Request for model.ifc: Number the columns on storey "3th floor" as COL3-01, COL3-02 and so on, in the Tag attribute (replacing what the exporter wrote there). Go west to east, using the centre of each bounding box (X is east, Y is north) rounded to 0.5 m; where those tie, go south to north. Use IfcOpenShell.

First a look at what the model holds.

```python
import ifcopenshell
import ifcopenshell.util.element
import ifcopenshell.util.placement

model = ifcopenshell.open("model.ifc")
print(model.schema)
storey = next(s for s in model.by_type("IfcBuildingStorey") if s.Name == "3th floor")
columns = [e for e in ifcopenshell.util.element.get_decomposition(storey) if e.is_a("IfcColumn")]
for e in sorted(columns, key=lambda e: e.id()):
    origin = ifcopenshell.util.placement.get_local_placement(e.ObjectPlacement)[:3, 3]
    print(e.id(), e.Tag, e.Name, origin.round(2) + 0.0, sep=" | ")
```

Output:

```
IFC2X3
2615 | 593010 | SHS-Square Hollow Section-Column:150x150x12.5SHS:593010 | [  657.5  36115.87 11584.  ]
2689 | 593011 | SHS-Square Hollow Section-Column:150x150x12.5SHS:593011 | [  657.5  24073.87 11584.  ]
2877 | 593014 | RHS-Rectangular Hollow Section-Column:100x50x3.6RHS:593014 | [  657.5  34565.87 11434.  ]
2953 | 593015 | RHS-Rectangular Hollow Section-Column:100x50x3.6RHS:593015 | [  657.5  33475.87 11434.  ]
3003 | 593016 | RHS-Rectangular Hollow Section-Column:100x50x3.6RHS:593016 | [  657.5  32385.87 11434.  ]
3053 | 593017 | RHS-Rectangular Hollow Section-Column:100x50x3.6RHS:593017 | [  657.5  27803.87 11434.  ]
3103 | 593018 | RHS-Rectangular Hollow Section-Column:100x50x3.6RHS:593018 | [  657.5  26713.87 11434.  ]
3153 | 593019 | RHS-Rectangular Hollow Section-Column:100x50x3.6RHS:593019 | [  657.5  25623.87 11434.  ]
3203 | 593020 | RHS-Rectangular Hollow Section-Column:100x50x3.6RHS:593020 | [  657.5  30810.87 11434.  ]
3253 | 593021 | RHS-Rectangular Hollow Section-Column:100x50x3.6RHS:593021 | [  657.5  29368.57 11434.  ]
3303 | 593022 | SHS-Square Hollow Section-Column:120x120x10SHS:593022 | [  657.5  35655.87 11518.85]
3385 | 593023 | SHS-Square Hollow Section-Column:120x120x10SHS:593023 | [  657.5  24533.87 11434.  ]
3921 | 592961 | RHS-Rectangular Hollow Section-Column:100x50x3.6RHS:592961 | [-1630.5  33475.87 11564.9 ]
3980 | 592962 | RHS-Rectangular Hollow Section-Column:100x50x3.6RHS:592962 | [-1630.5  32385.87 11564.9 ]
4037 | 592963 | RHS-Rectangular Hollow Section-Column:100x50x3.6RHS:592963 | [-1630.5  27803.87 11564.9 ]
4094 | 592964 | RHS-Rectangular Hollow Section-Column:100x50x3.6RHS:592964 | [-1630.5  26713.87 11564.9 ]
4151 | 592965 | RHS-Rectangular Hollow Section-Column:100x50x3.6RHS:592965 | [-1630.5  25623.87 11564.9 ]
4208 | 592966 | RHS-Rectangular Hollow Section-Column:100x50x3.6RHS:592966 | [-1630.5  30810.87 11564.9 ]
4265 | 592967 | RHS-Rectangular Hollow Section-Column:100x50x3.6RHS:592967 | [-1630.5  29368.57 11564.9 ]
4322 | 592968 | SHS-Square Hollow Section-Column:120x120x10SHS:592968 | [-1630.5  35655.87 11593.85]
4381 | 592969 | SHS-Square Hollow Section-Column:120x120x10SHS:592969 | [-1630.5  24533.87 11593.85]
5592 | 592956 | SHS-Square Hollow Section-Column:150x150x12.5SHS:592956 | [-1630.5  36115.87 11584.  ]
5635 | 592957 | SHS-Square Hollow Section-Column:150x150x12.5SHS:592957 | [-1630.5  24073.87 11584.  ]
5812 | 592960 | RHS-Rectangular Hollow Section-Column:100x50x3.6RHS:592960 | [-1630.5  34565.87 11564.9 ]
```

```python
import ifcopenshell
import ifcopenshell.geom
import ifcopenshell.util.element
import ifcopenshell.util.shape

model = ifcopenshell.open("model.ifc")
settings = ifcopenshell.geom.settings()
settings.set("use-world-coords", True)


def centre(element):
    shape = ifcopenshell.geom.create_shape(settings, element)
    return ifcopenshell.util.shape.get_bbox_centroid(shape.geometry)


storey = next(s for s in model.by_type("IfcBuildingStorey") if s.Name == "3th floor")
columns = [e for e in ifcopenshell.util.element.get_decomposition(storey) if e.is_a("IfcColumn")]

# Insertion points can sit at a corner or the storey origin, so sort by the geometry (in metres).
centres = {e: centre(e) for e in columns}
columns.sort(key=lambda e: (round(centres[e][0] / 0.5), centres[e][1]))

for i, e in enumerate(columns, start=1):
    number = f"COL3-{i:02d}"
    e.Tag = number
    print(e.id(), number)

model.write("model_v2.ifc")
```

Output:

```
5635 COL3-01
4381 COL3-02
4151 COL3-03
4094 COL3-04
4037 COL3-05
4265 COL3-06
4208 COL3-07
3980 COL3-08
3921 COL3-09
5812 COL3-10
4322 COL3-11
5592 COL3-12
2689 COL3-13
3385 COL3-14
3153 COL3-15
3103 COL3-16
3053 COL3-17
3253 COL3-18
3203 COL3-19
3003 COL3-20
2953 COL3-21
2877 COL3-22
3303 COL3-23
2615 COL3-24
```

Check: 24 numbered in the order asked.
